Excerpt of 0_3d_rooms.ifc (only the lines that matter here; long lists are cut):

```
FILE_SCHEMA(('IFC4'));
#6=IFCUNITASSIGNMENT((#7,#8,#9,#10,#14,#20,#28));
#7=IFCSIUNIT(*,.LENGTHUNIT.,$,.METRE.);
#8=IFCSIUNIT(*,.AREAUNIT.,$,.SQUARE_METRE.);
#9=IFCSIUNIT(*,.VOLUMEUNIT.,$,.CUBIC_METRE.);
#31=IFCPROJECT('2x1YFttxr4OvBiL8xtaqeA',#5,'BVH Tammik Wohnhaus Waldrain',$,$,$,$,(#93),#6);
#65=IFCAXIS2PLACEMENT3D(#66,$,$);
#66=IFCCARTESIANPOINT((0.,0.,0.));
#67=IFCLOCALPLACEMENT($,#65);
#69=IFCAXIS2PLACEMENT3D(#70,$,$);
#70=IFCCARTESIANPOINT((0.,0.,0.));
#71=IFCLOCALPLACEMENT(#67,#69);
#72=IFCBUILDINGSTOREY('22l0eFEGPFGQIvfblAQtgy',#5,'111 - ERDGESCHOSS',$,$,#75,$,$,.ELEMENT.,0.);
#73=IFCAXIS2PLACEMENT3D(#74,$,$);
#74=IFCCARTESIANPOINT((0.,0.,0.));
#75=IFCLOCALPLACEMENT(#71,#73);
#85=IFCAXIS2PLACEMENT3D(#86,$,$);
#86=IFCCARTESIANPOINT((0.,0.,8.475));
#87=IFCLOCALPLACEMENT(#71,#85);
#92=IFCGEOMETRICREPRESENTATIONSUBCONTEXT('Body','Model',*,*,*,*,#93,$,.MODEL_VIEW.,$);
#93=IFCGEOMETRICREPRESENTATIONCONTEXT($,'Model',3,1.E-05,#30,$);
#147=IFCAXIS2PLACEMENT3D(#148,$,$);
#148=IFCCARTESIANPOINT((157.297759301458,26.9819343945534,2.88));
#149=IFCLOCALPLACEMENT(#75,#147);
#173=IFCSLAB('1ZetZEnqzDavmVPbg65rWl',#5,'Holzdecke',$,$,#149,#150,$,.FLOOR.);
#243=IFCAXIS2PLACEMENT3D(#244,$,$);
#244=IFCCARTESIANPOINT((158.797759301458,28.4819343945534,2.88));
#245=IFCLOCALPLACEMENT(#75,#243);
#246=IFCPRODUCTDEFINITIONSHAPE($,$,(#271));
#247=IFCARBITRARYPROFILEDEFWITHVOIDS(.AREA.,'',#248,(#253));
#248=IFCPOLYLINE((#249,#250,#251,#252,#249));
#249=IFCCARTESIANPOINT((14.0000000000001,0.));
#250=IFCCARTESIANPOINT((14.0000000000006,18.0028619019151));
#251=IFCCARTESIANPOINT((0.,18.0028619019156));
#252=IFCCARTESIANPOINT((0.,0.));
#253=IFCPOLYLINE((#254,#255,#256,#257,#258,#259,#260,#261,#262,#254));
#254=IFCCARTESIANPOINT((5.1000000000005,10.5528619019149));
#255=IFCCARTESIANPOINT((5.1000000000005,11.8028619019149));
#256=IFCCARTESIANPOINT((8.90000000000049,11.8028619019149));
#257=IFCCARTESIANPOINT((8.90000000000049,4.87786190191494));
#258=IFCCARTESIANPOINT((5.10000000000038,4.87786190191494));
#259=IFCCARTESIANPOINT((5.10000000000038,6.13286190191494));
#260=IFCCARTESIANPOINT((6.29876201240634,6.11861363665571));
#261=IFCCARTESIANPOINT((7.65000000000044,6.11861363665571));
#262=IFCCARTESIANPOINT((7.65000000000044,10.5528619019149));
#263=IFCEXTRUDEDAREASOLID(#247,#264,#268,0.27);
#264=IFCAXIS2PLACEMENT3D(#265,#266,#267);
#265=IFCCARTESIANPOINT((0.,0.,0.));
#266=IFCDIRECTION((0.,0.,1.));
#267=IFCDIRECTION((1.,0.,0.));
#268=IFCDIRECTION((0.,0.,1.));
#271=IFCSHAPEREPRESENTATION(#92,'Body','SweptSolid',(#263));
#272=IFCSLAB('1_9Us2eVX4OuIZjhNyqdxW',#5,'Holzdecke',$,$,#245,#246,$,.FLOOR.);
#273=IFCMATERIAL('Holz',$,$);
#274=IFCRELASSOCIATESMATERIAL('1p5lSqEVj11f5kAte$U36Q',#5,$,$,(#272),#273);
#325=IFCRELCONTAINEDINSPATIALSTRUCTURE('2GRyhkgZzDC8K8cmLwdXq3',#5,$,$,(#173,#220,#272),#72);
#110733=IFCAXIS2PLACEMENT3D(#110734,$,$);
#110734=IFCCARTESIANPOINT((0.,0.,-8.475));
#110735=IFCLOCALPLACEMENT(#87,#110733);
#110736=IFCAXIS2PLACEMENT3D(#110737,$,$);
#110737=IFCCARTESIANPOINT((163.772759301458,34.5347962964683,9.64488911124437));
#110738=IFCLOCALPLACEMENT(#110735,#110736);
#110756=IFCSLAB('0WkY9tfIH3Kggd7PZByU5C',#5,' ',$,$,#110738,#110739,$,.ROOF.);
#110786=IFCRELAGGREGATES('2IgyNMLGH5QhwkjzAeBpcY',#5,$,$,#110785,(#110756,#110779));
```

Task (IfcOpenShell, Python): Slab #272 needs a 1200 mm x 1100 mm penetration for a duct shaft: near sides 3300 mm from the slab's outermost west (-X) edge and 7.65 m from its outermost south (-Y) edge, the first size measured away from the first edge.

```python
import numpy as np
import ifcopenshell
import ifcopenshell.api.feature
import ifcopenshell.api.geometry
import ifcopenshell.api.root
import ifcopenshell.geom
import ifcopenshell.util.placement
import ifcopenshell.util.representation
import ifcopenshell.util.shape
import ifcopenshell.util.unit

model = ifcopenshell.open("0_3d_rooms.ifc")
unit_scale = ifcopenshell.util.unit.calculate_unit_scale(model)
settings = ifcopenshell.geom.settings()


def volume(element):
    """Net volume in cubic metres, openings subtracted."""
    shape = ifcopenshell.geom.create_shape(settings, element)
    return ifcopenshell.util.shape.get_volume(shape.geometry)


slab = model.by_guid("1_9Us2eVX4OuIZjhNyqdxW")
before = volume(slab)

# Extent in the slab's own axes, in metres. The edges named are its -X and -Y sides.
slab_shape = ifcopenshell.geom.create_shape(settings, slab)
vertices = ifcopenshell.util.shape.get_vertices(slab_shape.geometry)
x_min, y_min, bottom = vertices.min(axis=0)
top = vertices[:, 2].max()

opening = ifcopenshell.api.root.create_entity(model, ifc_class="IfcOpeningElement", name="Duct shaft opening", predefined_type="OPENING")
context = ifcopenshell.util.representation.get_context(model, "Model", "Body", "MODEL_VIEW")
width, depth = 1.2, 1.1
outline = [(0.0, 0.0), (width, 0.0), (width, depth), (0.0, depth), (0.0, 0.0)]
# Overshoot both faces by 50 mm so the cut is clean.
shape = ifcopenshell.api.geometry.add_slab_representation(
    model, context=context, depth=top - bottom + 0.1, polyline=outline
)
ifcopenshell.api.geometry.assign_representation(model, product=opening, representation=shape)

matrix = ifcopenshell.util.placement.get_local_placement(slab.ObjectPlacement)
matrix[:, 3] = matrix @ np.append(np.array([x_min + 3.3, y_min + 7.65, bottom - 0.05]) / unit_scale, 1.0)
ifcopenshell.api.geometry.edit_object_placement(model, product=opening, matrix=matrix, is_si=False)
ifcopenshell.api.feature.add_feature(model, feature=opening, element=slab)

after = volume(slab)

print(f"slab volume {before:.3f} -> {after:.3f} m3")

model.write("0_3d_rooms-out.ifc")
```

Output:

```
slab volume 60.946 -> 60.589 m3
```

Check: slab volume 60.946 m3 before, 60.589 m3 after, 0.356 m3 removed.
